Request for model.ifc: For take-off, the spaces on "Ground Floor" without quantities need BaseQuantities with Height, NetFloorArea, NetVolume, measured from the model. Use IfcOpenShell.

First a look at what the model holds.

```python
import ifcopenshell
import ifcopenshell.util.element
import ifcopenshell.util.unit

model = ifcopenshell.open("model.ifc")
print(model.schema)
for unit_type in ("LENGTHUNIT", "AREAUNIT", "VOLUMEUNIT"):
    print(unit_type, ifcopenshell.util.unit.calculate_unit_scale(model, unit_type))
storey = next(s for s in model.by_type("IfcBuildingStorey") if s.Name == "Ground Floor")
spaces = [e for e in ifcopenshell.util.element.get_decomposition(storey) if e.is_a("IfcSpace")]
for e in sorted(spaces, key=lambda e: e.id()):
    print(e.id(), e.is_a(), e.Name, list(ifcopenshell.util.element.get_psets(e, qtos_only=True)), sep=" | ")
```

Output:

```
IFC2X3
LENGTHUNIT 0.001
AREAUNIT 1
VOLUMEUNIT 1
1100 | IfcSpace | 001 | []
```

```python
import ifcopenshell
import ifcopenshell.api.pset
import ifcopenshell.geom
import ifcopenshell.util.element
import ifcopenshell.util.shape
import ifcopenshell.util.unit

model = ifcopenshell.open("model.ifc")
unit_scale = ifcopenshell.util.unit.calculate_unit_scale(model)
area_scale = ifcopenshell.util.unit.calculate_unit_scale(model, "AREAUNIT")
volume_scale = ifcopenshell.util.unit.calculate_unit_scale(model, "VOLUMEUNIT")
settings = ifcopenshell.geom.settings()

storey = next(s for s in model.by_type("IfcBuildingStorey") if s.Name == "Ground Floor")
spaces = [e for e in ifcopenshell.util.element.get_decomposition(storey) if e.is_a("IfcSpace")]

for e in sorted(spaces, key=lambda e: e.id()):
    if ifcopenshell.util.element.get_psets(e, qtos_only=True, should_inherit=False):
        continue
    # Geometry comes back in metres, in the element's own axes.
    shape = ifcopenshell.geom.create_shape(settings, e)
    values = {
        "Height": ifcopenshell.util.shape.get_z(shape.geometry) / unit_scale,
        "NetFloorArea": ifcopenshell.util.shape.get_footprint_area(shape.geometry) / area_scale,
        "NetVolume": ifcopenshell.util.shape.get_volume(shape.geometry) / volume_scale,
    }
    qto = ifcopenshell.api.pset.add_qto(model, product=e, name="BaseQuantities")
    ifcopenshell.api.pset.edit_qto(model, qto=qto, properties=values)
    print(e.id(), {k: round(v, 3) for k, v in values.items()})

model.write("model_rev.ifc")
```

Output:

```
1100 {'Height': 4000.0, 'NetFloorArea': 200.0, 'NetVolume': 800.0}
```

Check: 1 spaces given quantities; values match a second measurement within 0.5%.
